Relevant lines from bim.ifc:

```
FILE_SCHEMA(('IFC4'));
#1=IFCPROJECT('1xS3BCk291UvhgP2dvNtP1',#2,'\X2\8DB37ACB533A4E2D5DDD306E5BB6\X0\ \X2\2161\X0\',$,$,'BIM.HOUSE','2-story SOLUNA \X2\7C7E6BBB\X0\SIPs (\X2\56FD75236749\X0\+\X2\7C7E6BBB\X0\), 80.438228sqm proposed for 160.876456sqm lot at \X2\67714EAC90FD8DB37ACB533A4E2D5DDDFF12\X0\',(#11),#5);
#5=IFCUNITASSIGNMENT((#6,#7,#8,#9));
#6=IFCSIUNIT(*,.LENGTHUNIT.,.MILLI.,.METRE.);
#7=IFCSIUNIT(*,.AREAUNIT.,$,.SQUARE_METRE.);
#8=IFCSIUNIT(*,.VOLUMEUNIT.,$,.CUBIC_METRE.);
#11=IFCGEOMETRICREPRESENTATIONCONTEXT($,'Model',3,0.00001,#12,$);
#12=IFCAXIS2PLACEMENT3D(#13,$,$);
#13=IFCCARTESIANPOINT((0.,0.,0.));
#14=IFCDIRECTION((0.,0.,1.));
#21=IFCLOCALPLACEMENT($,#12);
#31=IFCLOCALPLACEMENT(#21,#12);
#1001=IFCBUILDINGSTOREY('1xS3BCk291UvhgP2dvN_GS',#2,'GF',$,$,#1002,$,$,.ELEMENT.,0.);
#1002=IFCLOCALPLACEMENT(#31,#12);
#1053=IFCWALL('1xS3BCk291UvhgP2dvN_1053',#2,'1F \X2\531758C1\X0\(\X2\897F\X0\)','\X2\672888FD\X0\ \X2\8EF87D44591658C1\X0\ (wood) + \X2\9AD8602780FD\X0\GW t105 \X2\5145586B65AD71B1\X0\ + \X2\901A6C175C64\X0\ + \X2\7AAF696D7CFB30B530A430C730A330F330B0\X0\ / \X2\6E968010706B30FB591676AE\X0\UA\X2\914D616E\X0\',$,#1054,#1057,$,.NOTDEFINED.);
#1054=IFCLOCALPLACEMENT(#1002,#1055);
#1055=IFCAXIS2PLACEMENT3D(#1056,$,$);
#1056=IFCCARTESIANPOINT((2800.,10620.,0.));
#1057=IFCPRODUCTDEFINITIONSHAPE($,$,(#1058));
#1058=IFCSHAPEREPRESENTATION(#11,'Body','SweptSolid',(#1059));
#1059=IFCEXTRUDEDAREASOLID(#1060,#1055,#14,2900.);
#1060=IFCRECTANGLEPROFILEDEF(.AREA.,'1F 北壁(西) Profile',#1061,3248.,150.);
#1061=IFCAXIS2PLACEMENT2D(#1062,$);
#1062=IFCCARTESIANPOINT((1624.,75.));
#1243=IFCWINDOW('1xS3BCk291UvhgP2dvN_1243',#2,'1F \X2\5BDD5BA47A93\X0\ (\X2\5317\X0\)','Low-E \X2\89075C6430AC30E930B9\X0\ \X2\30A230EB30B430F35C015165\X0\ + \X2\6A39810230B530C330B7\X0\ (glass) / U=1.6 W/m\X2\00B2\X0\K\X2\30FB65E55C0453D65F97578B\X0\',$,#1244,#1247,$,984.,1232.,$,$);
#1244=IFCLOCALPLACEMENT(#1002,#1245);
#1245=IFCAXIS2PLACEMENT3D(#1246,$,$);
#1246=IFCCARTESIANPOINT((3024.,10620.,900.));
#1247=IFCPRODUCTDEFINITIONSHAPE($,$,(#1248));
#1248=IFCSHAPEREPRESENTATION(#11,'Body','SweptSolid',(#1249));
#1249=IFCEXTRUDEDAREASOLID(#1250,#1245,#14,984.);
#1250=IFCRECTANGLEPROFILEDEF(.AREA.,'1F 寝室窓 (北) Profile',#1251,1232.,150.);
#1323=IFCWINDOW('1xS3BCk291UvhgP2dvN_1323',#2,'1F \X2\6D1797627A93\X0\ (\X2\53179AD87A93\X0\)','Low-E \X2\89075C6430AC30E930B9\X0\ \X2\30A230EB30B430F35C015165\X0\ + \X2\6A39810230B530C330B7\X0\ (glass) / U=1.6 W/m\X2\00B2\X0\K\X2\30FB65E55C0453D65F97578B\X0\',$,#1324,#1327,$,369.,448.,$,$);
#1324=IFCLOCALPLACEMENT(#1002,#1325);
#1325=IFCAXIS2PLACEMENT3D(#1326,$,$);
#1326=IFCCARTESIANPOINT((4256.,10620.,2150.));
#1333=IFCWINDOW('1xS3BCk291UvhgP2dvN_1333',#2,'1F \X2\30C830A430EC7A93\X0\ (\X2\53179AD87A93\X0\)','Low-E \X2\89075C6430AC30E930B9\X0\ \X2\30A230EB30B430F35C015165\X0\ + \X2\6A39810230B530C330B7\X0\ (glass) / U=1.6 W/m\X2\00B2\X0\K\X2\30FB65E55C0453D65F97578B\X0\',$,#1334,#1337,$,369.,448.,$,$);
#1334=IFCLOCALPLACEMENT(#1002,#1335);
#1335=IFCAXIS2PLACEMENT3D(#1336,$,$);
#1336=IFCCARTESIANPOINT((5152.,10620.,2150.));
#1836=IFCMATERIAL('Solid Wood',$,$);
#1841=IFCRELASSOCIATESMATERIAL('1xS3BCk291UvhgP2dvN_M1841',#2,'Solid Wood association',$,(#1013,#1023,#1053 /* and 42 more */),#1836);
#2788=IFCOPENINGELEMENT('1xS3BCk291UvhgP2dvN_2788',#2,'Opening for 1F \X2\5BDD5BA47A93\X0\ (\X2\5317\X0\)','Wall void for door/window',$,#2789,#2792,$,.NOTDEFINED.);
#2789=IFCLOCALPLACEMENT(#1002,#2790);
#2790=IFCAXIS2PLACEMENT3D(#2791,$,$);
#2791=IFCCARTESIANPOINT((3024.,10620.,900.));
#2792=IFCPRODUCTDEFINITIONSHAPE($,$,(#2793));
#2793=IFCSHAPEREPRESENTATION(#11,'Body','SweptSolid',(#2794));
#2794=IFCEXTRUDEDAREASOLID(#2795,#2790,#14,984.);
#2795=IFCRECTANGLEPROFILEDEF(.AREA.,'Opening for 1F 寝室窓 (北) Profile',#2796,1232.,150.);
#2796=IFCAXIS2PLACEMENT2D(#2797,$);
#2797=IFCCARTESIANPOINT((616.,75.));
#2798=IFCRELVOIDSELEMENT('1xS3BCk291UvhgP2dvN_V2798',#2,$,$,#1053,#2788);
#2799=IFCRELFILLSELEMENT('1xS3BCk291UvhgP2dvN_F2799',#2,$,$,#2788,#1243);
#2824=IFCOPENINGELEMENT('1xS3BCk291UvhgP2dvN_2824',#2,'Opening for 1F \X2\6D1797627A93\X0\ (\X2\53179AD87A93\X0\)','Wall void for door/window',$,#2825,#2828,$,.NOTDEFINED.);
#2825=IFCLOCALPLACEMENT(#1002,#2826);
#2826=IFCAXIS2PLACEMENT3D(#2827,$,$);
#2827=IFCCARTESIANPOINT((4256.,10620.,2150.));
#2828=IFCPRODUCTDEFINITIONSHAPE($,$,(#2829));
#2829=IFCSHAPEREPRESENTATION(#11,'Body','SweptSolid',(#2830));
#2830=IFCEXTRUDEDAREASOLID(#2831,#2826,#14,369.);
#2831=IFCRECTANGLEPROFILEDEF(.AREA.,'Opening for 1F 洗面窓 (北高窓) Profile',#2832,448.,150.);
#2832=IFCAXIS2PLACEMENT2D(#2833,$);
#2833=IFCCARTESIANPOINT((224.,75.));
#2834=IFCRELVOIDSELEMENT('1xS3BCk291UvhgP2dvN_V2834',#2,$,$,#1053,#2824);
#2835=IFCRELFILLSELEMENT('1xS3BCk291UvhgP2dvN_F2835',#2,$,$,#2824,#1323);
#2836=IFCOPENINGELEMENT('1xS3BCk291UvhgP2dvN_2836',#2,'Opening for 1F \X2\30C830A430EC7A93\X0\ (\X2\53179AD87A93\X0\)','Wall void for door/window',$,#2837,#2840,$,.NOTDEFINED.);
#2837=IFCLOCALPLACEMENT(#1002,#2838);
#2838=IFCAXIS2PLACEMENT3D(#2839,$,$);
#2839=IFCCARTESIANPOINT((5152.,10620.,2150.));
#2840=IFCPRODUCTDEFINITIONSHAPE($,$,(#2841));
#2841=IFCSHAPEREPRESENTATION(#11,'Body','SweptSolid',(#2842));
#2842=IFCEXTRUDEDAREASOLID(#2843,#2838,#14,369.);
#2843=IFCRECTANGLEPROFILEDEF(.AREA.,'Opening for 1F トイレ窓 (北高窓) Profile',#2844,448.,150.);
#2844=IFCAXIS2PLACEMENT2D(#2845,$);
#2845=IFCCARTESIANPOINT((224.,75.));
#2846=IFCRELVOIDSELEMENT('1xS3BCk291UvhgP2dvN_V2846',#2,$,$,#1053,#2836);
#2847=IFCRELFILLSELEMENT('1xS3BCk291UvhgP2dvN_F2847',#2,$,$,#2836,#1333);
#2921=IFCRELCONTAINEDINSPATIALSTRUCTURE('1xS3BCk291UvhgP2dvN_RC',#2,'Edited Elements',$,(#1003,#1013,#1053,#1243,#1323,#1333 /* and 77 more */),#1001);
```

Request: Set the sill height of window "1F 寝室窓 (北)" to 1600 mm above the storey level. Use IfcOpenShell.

```python
import numpy as np
import ifcopenshell
import ifcopenshell.api.geometry
import ifcopenshell.geom
import ifcopenshell.util.element
import ifcopenshell.util.placement
import ifcopenshell.util.shape
import ifcopenshell.util.unit

model = ifcopenshell.open("bim.ifc")
unit_scale = ifcopenshell.util.unit.calculate_unit_scale(model)

window = model.by_id(1243)
opening = window.FillsVoids[0].RelatingOpeningElement
storey = ifcopenshell.util.element.get_container(window, ifc_class="IfcBuildingStorey")
level = ifcopenshell.util.placement.get_local_placement(storey.ObjectPlacement)[2, 3]

# The opening's origin need not be at the sill, so measure its lowest point.
shape = ifcopenshell.geom.create_shape(ifcopenshell.geom.settings(), opening)
bottom = ifcopenshell.util.shape.get_shape_bottom_elevation(shape, shape.geometry) / unit_scale
dz = level + 1600.0 - bottom

shift = np.array([0.0, 0.0, dz])
# The window is not placed relative to its opening, so move both.
for product in (opening, window):
    matrix = ifcopenshell.util.placement.get_local_placement(product.ObjectPlacement)
    matrix[:3, 3] += shift
    ifcopenshell.api.geometry.edit_object_placement(model, product=product, matrix=matrix, is_si=False)

print(f"moved by {dz * unit_scale:+.3f} m")

model.write("bim_rev.ifc")
```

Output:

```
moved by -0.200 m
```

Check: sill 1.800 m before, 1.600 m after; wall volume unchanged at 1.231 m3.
